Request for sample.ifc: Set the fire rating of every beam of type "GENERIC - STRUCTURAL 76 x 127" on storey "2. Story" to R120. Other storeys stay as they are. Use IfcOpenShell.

First a look at what the model holds.

```python
import ifcopenshell
import ifcopenshell.util.element

model = ifcopenshell.open("sample.ifc")
print(model.schema)
storey = next(s for s in model.by_type("IfcBuildingStorey") if s.Name == "2. Story")
beams = [e for e in ifcopenshell.util.element.get_decomposition(storey) if e.is_a("IfcBeam")]
seen = {}
for e in beams:
    element_type = ifcopenshell.util.element.get_type(e)
    key = (element_type.Name if element_type != e and element_type else None, ifcopenshell.util.element.get_pset(e, "Pset_BeamCommon", "FireRating"))
    seen[key] = seen.get(key, 0) + 1
for (name, value), count in sorted(seen.items(), key=str):
    print(count, "x", name, "|", value)
```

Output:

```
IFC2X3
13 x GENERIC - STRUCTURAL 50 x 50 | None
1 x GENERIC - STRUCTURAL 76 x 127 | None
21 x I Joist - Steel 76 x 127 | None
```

```python
import ifcopenshell
import ifcopenshell.api.pset
import ifcopenshell.util.element

model = ifcopenshell.open("sample.ifc")

storey = next(s for s in model.by_type("IfcBuildingStorey") if s.Name == "2. Story")
beams = [e for e in ifcopenshell.util.element.get_decomposition(storey) if e.is_a("IfcBeam")]

count = 0
for e in beams:
    element_type = ifcopenshell.util.element.get_type(e)
    if element_type in (None, e) or element_type.Name != "GENERIC - STRUCTURAL 76 x 127":
        continue
    # add_pset returns the element's existing set when there is one.
    pset = ifcopenshell.api.pset.add_pset(model, product=e, name="Pset_BeamCommon")
    ifcopenshell.api.pset.edit_pset(model, pset=pset, properties={"FireRating": "R120"})
    count += 1

print(count, "beams updated")

model.write("sample_v2.ifc")
```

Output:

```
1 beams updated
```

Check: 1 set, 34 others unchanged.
